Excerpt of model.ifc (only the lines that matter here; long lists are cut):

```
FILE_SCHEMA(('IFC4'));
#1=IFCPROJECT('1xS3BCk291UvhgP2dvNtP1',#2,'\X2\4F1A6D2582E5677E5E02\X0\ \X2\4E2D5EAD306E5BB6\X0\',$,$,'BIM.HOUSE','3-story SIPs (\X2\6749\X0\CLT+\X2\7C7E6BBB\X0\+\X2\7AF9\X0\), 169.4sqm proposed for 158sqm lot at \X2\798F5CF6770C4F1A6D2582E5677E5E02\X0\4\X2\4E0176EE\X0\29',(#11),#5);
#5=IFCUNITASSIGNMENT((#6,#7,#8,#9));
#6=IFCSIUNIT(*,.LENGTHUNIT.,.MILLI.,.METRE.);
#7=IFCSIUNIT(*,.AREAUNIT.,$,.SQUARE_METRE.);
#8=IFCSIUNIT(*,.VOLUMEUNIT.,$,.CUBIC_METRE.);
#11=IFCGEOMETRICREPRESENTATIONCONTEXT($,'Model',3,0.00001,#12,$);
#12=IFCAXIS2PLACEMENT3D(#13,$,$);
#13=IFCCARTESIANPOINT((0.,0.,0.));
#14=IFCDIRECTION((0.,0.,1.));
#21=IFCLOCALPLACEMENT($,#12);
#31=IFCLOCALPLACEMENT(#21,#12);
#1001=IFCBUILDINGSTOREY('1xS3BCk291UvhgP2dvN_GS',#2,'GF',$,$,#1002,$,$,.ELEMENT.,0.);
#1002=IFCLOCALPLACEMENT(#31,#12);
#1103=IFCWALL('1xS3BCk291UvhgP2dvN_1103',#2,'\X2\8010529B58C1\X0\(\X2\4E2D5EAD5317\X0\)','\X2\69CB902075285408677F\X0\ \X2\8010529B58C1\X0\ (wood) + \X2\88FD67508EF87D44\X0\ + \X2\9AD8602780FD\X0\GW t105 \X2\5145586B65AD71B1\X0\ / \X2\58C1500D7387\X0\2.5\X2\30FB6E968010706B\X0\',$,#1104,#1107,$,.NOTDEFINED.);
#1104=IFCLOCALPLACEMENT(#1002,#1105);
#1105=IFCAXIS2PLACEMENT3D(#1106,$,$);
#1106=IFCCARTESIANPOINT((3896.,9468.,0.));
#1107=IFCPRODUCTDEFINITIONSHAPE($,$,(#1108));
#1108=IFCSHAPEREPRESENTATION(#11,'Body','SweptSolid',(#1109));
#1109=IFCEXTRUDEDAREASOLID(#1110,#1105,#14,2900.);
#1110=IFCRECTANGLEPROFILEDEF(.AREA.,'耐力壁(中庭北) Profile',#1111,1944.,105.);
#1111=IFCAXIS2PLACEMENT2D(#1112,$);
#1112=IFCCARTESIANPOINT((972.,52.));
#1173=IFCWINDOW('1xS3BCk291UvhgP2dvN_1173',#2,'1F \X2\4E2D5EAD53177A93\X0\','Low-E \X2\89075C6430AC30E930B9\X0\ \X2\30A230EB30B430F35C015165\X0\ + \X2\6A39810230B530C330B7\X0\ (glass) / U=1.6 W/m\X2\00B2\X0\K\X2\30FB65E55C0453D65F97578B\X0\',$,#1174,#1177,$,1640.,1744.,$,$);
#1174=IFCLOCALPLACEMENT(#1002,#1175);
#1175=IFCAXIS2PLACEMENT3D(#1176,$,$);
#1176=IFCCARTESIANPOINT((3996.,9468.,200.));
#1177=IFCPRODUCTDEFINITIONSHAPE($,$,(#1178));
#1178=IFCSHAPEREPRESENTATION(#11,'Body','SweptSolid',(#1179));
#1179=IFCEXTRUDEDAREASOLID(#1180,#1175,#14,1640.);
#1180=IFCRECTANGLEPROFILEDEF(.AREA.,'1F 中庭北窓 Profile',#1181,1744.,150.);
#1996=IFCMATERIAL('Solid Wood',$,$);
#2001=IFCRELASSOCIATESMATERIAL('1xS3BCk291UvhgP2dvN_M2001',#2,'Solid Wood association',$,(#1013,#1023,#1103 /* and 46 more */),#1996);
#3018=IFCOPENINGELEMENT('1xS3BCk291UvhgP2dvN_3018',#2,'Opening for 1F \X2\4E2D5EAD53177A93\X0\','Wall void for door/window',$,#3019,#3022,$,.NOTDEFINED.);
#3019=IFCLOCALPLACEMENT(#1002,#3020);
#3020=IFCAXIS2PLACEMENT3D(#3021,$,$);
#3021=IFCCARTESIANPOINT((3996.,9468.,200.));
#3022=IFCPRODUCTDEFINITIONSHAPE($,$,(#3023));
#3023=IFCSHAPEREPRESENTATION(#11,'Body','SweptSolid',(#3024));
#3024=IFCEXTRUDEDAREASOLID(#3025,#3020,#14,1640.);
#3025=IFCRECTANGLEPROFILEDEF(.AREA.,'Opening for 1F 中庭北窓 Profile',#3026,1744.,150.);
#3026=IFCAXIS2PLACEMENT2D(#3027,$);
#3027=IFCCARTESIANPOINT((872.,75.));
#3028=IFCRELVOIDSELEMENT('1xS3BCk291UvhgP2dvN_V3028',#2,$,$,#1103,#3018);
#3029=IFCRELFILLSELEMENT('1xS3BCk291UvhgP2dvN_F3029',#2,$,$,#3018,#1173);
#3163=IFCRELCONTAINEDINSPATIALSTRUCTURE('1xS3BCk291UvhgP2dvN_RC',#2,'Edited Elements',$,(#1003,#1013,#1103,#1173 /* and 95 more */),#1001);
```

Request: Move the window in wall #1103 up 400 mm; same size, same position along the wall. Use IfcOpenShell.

```python
import numpy as np
import ifcopenshell
import ifcopenshell.api.geometry
import ifcopenshell.util.placement
import ifcopenshell.util.unit

model = ifcopenshell.open("model.ifc")
unit_scale = ifcopenshell.util.unit.calculate_unit_scale(model)

window = model.by_guid("1xS3BCk291UvhgP2dvN_1173")
opening = window.FillsVoids[0].RelatingOpeningElement
dz = 400.0

shift = np.array([0.0, 0.0, dz])
# The window is not placed relative to its opening, so move both.
for product in (opening, window):
    matrix = ifcopenshell.util.placement.get_local_placement(product.ObjectPlacement)
    matrix[:3, 3] += shift
    ifcopenshell.api.geometry.edit_object_placement(model, product=product, matrix=matrix, is_si=False)

print(f"moved by {dz * unit_scale:+.3f} m")

model.write("model-out.ifc")
```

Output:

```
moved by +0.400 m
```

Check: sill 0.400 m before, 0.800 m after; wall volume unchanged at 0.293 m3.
